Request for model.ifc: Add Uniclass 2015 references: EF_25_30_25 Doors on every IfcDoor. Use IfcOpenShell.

First a look at what the model holds.

```python
import ifcopenshell

model = ifcopenshell.open("model.ifc")
print(model.schema)
print("classifications:", [c.Name for c in model.by_type("IfcClassification")])
for ifc_class in ("IfcDoor", "IfcRoof", "IfcStair", "IfcWall", "IfcWindow"):
    print(ifc_class, len(model.by_type(ifc_class)))
```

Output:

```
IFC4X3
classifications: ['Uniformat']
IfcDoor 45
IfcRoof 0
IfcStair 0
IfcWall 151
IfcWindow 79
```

```python
import ifcopenshell
import ifcopenshell.api.classification

model = ifcopenshell.open("model.ifc")

system = ifcopenshell.api.classification.add_classification(model, classification="Uniclass 2015")

codes = {
    "IfcDoor": ("EF_25_30_25", "Doors"),
}
for ifc_class, (code, name) in codes.items():
    products = model.by_type(ifc_class)
    ifcopenshell.api.classification.add_reference(
        model, products=products, classification=system, identification=code, name=name
    )
    print(code, len(products))

model.write("model_rev.ifc")
```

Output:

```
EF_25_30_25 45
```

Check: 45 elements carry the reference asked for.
